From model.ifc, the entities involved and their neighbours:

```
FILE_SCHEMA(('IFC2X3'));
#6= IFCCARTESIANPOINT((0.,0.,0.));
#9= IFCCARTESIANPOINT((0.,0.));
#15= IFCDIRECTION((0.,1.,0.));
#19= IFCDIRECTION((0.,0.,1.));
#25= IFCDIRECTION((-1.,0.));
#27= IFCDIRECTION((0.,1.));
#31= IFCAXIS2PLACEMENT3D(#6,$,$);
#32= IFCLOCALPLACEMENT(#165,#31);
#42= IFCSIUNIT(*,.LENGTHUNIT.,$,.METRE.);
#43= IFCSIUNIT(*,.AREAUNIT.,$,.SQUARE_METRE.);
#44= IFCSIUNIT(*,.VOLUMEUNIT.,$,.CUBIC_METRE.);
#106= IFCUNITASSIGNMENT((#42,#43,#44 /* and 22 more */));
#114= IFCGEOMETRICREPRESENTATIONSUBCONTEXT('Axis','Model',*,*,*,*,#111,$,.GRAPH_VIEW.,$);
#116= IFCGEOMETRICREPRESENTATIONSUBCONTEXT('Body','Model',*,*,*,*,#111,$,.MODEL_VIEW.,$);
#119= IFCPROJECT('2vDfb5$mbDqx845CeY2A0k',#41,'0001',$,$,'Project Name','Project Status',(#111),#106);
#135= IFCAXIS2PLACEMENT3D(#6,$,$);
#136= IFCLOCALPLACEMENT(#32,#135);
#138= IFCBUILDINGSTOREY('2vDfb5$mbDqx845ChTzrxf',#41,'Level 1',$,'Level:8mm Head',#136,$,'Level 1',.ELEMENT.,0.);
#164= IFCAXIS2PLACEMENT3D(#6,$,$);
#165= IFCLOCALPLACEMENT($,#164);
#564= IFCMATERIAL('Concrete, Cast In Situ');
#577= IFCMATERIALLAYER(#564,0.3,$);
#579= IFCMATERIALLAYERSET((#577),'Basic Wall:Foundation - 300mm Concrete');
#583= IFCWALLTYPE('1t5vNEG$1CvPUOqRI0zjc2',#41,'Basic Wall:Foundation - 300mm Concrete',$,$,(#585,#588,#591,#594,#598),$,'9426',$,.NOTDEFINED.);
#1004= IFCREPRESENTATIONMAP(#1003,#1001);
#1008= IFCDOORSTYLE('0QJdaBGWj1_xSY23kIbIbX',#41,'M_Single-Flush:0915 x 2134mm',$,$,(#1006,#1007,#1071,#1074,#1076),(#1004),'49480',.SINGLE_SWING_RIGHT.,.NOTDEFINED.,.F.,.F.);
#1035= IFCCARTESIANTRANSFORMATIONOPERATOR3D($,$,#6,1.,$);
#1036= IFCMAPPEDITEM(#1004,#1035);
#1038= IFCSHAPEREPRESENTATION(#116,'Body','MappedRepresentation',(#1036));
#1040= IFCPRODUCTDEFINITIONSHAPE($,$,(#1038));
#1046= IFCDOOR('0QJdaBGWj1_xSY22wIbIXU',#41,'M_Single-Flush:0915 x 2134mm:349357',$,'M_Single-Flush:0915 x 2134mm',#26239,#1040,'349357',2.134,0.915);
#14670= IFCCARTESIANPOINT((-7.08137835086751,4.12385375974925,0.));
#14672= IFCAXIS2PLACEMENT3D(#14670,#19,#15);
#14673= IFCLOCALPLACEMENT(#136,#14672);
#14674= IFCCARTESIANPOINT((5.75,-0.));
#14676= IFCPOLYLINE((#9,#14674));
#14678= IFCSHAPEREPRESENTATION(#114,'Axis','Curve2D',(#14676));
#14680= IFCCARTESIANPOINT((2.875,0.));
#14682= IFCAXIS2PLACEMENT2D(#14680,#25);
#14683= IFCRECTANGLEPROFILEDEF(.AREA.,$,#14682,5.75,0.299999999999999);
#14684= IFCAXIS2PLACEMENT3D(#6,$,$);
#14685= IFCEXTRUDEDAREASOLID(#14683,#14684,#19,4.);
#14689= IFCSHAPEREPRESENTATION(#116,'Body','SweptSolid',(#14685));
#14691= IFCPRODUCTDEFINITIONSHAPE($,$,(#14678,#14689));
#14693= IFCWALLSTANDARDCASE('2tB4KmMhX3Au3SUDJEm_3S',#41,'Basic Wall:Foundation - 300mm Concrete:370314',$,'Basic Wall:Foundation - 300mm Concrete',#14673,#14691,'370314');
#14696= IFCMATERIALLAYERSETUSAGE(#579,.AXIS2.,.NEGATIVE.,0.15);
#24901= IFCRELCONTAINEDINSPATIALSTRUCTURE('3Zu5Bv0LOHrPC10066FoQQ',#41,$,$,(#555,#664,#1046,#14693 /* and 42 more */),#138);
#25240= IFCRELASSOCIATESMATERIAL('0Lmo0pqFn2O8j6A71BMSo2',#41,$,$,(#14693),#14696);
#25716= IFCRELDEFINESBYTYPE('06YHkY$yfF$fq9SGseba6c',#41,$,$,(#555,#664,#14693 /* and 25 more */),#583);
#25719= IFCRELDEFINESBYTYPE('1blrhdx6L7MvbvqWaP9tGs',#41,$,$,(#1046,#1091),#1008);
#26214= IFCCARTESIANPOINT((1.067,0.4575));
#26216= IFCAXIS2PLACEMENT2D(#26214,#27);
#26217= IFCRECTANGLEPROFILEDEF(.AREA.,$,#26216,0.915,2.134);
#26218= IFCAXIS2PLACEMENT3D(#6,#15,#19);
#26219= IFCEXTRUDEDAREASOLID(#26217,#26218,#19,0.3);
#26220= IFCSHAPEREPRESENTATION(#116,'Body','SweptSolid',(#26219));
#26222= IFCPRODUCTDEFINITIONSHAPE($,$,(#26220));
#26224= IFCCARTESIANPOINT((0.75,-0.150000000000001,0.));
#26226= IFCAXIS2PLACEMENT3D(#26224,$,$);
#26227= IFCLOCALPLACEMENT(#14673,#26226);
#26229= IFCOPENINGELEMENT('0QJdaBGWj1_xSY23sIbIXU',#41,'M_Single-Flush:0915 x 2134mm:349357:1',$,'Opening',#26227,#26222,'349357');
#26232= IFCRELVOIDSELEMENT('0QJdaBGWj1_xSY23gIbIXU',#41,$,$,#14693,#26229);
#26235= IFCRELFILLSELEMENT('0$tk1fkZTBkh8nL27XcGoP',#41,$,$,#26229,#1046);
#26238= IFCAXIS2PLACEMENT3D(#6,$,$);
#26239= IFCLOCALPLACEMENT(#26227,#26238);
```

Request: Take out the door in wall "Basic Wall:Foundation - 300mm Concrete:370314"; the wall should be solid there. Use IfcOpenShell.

```python
import ifcopenshell
import ifcopenshell.api.feature
import ifcopenshell.api.root
import ifcopenshell.geom
import ifcopenshell.util.shape

model = ifcopenshell.open("model.ifc")
settings = ifcopenshell.geom.settings()


def volume(element):
    """Net volume in cubic metres, openings subtracted."""
    shape = ifcopenshell.geom.create_shape(settings, element)
    return ifcopenshell.util.shape.get_volume(shape.geometry)


door = model.by_guid("0QJdaBGWj1_xSY22wIbIXU")
opening = door.FillsVoids[0].RelatingOpeningElement
wall = opening.VoidsElements[0].RelatingBuildingElement
before = volume(wall)

ifcopenshell.api.root.remove_product(model, product=door)
ifcopenshell.api.feature.remove_feature(model, feature=opening)

after = volume(wall)

print(f"wall volume {before:.3f} -> {after:.3f} m3")

model.write("model_rev.ifc")
```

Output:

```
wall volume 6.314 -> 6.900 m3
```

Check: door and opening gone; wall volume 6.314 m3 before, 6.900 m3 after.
